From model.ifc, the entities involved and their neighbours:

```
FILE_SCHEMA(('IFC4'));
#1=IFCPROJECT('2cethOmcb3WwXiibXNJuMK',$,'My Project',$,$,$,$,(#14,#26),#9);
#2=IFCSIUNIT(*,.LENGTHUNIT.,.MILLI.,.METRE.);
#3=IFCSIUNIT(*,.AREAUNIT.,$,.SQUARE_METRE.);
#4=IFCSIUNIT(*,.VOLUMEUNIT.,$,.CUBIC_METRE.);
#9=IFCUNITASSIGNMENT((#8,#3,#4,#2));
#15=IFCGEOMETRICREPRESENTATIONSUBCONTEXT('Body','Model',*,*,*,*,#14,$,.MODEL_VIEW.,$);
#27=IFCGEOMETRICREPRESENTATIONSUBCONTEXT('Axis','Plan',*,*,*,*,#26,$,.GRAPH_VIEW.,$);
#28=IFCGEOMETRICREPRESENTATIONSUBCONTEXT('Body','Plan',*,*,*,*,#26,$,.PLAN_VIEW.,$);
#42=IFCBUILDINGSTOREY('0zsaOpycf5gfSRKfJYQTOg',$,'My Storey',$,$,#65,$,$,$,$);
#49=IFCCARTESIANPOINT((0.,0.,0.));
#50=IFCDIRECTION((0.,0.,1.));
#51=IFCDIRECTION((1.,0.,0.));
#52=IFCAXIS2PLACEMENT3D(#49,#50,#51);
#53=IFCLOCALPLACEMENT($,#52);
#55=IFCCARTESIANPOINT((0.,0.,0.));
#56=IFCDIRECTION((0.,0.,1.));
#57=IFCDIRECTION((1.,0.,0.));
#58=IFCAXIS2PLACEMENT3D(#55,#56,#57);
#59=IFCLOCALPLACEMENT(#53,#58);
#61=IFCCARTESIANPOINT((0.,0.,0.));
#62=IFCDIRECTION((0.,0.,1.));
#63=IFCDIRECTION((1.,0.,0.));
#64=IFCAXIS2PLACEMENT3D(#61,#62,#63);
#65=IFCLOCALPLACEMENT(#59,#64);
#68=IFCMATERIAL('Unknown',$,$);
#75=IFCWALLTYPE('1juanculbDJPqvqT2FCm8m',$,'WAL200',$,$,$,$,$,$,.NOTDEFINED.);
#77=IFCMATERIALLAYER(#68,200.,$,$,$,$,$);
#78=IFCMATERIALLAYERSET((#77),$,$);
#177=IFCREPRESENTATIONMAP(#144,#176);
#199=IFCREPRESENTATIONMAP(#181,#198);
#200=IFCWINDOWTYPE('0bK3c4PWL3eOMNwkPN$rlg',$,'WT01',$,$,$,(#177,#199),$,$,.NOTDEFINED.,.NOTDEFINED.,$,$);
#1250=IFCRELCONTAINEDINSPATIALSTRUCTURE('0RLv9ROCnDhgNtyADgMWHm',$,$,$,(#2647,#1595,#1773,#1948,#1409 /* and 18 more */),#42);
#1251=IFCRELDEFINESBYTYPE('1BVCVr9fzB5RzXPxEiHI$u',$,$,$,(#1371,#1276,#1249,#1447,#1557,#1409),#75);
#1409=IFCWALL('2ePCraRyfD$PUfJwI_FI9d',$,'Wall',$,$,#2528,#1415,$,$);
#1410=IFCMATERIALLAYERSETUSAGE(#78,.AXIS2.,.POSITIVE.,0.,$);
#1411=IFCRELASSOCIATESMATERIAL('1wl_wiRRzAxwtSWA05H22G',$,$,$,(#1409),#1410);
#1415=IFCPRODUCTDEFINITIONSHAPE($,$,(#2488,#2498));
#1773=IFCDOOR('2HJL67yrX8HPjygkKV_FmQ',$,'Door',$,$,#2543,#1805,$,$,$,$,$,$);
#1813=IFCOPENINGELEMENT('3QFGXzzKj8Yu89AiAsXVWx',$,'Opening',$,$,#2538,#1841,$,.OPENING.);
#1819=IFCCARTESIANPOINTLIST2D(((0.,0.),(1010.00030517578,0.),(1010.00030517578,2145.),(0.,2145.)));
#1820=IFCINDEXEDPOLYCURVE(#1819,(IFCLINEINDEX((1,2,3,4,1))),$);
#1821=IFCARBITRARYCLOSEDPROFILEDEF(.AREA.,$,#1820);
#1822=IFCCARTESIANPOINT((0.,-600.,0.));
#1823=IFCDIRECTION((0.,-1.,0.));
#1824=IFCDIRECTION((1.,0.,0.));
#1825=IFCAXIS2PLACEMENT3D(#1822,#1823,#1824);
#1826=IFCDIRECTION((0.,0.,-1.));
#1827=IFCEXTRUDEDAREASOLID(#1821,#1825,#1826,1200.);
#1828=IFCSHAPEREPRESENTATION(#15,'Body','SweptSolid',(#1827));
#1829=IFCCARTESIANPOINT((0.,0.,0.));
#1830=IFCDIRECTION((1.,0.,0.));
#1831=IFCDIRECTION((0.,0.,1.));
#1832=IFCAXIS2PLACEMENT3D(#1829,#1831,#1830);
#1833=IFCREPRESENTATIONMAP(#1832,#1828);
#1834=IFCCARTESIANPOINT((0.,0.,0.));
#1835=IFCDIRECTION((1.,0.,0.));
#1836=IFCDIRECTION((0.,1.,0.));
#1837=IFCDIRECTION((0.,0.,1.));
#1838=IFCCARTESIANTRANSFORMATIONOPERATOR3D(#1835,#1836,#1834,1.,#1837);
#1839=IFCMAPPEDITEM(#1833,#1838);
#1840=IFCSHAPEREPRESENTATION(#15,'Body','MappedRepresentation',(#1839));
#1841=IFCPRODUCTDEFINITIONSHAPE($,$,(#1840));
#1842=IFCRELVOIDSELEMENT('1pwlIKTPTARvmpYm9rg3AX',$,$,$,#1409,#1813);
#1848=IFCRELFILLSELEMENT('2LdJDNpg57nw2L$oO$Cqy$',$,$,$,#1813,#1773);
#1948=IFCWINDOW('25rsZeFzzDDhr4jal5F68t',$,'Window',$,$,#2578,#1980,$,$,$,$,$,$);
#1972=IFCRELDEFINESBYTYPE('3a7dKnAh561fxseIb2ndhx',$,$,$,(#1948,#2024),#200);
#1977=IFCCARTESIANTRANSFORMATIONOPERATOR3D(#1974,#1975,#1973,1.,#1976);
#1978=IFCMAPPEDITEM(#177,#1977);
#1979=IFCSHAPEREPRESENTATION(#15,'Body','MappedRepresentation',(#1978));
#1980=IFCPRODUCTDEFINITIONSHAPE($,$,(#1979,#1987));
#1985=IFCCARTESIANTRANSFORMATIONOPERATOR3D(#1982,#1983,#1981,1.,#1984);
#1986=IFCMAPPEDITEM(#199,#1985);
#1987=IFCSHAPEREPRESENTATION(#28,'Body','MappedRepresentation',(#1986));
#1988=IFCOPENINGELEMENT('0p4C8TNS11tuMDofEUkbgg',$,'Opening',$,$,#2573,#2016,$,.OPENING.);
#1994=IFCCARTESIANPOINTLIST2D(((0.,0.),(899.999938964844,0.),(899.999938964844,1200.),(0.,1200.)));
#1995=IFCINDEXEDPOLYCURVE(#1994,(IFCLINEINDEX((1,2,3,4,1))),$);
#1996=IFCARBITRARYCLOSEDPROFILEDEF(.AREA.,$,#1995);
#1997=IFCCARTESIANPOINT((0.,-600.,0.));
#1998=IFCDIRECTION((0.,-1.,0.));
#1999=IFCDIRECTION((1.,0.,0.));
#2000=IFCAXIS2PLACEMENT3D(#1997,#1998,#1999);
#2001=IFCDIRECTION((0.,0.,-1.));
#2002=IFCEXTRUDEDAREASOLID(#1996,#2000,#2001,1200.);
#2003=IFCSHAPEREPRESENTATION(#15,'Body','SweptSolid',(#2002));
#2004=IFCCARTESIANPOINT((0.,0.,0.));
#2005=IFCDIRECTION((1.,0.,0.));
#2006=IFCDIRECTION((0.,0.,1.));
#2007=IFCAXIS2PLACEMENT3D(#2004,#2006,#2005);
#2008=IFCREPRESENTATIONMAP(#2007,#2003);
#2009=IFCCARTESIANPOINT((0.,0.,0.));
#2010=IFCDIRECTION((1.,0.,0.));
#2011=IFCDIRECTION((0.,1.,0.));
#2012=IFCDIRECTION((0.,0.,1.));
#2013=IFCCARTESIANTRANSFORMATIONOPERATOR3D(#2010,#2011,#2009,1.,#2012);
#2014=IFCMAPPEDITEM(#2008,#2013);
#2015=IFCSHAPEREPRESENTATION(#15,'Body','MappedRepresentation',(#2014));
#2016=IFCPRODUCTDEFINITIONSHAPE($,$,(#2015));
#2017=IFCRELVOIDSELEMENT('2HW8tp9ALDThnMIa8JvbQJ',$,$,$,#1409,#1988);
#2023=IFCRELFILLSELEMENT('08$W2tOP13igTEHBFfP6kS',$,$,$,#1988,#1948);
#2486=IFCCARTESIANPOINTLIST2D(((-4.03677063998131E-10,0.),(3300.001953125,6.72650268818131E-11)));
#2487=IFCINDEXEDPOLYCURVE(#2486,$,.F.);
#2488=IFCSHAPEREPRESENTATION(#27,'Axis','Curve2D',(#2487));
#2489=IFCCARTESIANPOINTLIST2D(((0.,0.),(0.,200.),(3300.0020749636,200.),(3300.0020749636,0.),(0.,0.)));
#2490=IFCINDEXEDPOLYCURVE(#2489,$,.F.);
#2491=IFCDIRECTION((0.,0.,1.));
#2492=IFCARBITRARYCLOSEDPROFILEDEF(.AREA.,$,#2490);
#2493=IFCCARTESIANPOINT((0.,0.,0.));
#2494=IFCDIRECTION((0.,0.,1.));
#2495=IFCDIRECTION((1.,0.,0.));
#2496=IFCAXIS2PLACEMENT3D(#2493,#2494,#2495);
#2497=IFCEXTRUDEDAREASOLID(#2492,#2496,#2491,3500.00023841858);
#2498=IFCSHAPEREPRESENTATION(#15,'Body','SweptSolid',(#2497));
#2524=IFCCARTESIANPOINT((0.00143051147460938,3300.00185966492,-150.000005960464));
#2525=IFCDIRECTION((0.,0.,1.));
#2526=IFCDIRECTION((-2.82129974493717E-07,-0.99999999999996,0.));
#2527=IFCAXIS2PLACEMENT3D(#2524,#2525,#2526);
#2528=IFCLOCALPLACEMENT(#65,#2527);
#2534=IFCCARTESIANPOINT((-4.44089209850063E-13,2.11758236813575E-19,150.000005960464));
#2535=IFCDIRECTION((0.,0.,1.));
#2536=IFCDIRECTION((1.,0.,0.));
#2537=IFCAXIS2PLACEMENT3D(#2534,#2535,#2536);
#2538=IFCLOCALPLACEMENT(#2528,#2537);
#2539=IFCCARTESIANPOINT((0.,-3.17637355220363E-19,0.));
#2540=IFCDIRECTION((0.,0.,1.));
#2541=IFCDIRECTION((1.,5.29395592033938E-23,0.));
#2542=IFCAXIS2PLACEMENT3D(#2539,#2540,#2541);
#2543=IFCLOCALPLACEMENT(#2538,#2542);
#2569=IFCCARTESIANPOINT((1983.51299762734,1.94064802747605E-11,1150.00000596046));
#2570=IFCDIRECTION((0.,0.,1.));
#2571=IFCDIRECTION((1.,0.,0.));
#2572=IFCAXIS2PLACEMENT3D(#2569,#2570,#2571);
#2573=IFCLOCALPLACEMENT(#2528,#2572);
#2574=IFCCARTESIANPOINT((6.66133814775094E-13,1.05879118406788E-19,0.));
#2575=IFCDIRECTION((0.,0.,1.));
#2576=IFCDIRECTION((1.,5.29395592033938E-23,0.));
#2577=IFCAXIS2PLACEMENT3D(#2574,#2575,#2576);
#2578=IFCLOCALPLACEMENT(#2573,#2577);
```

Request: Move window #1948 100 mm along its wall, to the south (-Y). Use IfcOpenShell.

```python
import ifcopenshell
import ifcopenshell.api.geometry
import ifcopenshell.util.placement

model = ifcopenshell.open("model.ifc")

window = model.by_id(1948)
opening = window.FillsVoids[0].RelatingOpeningElement
wall = opening.VoidsElements[0].RelatingBuildingElement

wall_matrix = ifcopenshell.util.placement.get_local_placement(wall.ObjectPlacement)
shift = wall_matrix[:3, 0] * 100.0
before = ifcopenshell.util.placement.get_local_placement(window.ObjectPlacement)[:3, 3].copy()

# The window is placed relative to its opening, so it follows when the opening moves.
matrix = ifcopenshell.util.placement.get_local_placement(opening.ObjectPlacement)
matrix[:3, 3] += shift
ifcopenshell.api.geometry.edit_object_placement(
    model, product=opening, matrix=matrix, is_si=False, should_transform_children=True
)

after = ifcopenshell.util.placement.get_local_placement(window.ObjectPlacement)[:3, 3]
print("window moved by", (after - before).round(3) + 0.0)

model.write("model_updated.ifc")
```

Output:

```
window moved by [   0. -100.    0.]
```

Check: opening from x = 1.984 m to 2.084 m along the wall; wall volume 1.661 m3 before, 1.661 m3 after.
